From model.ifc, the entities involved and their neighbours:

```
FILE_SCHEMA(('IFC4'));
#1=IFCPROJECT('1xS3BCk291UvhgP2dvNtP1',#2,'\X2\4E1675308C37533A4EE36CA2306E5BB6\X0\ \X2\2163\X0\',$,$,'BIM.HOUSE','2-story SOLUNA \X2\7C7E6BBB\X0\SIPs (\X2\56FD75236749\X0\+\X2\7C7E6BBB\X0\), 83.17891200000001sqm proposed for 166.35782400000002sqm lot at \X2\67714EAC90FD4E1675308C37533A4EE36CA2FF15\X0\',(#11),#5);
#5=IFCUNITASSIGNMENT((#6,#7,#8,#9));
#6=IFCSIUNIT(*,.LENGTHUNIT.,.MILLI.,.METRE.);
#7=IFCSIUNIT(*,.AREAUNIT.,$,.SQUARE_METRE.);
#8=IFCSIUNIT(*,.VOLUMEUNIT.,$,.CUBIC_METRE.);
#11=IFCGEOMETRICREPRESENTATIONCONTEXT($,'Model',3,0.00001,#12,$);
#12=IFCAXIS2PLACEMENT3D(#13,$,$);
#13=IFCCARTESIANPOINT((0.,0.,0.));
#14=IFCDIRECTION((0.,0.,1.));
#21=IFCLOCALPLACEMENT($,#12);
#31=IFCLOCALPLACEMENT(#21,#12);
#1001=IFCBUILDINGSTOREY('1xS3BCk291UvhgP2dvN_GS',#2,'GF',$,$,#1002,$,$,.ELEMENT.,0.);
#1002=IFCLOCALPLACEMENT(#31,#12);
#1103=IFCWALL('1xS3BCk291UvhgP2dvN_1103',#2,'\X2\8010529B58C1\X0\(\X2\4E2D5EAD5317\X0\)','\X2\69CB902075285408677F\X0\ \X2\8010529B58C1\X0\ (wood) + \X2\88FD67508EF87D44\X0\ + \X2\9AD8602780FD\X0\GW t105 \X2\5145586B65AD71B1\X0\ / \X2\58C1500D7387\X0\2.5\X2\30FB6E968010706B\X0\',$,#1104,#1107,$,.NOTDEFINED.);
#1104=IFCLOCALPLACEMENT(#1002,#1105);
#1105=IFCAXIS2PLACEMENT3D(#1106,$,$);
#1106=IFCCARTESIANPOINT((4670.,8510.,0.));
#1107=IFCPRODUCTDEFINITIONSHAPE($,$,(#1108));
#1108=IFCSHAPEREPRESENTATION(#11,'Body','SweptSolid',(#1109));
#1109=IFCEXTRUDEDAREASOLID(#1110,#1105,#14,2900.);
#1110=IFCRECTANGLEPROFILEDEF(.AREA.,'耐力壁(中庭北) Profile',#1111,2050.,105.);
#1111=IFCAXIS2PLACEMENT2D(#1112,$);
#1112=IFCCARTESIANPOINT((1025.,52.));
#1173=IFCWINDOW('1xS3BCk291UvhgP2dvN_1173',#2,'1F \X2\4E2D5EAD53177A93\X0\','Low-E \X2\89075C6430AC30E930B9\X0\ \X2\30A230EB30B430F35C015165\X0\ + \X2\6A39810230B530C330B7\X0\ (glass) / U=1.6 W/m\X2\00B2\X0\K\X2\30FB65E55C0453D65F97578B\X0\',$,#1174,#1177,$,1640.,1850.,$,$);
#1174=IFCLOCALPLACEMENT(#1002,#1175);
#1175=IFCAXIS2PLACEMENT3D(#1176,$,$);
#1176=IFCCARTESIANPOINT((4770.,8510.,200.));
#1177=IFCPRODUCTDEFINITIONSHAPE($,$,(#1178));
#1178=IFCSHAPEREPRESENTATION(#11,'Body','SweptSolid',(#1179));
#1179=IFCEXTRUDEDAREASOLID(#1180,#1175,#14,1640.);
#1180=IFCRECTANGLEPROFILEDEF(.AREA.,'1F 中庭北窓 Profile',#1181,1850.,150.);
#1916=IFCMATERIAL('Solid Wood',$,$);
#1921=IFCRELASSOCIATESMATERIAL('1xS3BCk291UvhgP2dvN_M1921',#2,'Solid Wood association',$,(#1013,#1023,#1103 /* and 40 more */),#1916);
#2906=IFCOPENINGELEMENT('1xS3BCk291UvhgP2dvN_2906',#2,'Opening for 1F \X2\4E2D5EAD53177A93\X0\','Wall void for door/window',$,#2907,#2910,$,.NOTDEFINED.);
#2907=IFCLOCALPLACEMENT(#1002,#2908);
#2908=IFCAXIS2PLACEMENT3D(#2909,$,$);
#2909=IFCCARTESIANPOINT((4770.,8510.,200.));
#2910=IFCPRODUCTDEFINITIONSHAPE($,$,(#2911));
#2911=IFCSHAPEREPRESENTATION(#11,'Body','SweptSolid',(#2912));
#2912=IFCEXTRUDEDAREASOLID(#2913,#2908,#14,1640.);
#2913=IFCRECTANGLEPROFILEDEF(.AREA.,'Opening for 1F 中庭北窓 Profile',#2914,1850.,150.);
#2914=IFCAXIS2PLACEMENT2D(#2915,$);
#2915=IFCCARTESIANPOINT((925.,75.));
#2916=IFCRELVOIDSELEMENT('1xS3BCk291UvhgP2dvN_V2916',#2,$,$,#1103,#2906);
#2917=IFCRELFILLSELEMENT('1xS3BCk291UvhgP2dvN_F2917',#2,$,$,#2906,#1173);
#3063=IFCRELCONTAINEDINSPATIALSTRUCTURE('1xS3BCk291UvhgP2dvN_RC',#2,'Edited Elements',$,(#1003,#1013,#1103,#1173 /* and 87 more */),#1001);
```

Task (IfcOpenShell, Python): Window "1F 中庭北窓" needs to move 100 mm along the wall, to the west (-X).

```python
import ifcopenshell
import ifcopenshell.api.geometry
import ifcopenshell.util.placement
import ifcopenshell.util.unit

model = ifcopenshell.open("model.ifc")
unit_scale = ifcopenshell.util.unit.calculate_unit_scale(model)

window = model.by_guid("1xS3BCk291UvhgP2dvN_1173")
opening = window.FillsVoids[0].RelatingOpeningElement
wall = opening.VoidsElements[0].RelatingBuildingElement

wall_matrix = ifcopenshell.util.placement.get_local_placement(wall.ObjectPlacement)
shift = wall_matrix[:3, 0] * -0.1 / unit_scale
before = ifcopenshell.util.placement.get_local_placement(window.ObjectPlacement)[:3, 3].copy()

# The window is not placed relative to its opening, so move both.
for product in (opening, window):
    matrix = ifcopenshell.util.placement.get_local_placement(product.ObjectPlacement)
    matrix[:3, 3] += shift
    ifcopenshell.api.geometry.edit_object_placement(model, product=product, matrix=matrix, is_si=False)

after = ifcopenshell.util.placement.get_local_placement(window.ObjectPlacement)[:3, 3]
print("window moved by", (after - before).round(3) + 0.0)

model.write("model_rev.ifc")
```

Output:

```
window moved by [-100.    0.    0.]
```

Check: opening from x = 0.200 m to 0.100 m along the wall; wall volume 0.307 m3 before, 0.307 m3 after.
